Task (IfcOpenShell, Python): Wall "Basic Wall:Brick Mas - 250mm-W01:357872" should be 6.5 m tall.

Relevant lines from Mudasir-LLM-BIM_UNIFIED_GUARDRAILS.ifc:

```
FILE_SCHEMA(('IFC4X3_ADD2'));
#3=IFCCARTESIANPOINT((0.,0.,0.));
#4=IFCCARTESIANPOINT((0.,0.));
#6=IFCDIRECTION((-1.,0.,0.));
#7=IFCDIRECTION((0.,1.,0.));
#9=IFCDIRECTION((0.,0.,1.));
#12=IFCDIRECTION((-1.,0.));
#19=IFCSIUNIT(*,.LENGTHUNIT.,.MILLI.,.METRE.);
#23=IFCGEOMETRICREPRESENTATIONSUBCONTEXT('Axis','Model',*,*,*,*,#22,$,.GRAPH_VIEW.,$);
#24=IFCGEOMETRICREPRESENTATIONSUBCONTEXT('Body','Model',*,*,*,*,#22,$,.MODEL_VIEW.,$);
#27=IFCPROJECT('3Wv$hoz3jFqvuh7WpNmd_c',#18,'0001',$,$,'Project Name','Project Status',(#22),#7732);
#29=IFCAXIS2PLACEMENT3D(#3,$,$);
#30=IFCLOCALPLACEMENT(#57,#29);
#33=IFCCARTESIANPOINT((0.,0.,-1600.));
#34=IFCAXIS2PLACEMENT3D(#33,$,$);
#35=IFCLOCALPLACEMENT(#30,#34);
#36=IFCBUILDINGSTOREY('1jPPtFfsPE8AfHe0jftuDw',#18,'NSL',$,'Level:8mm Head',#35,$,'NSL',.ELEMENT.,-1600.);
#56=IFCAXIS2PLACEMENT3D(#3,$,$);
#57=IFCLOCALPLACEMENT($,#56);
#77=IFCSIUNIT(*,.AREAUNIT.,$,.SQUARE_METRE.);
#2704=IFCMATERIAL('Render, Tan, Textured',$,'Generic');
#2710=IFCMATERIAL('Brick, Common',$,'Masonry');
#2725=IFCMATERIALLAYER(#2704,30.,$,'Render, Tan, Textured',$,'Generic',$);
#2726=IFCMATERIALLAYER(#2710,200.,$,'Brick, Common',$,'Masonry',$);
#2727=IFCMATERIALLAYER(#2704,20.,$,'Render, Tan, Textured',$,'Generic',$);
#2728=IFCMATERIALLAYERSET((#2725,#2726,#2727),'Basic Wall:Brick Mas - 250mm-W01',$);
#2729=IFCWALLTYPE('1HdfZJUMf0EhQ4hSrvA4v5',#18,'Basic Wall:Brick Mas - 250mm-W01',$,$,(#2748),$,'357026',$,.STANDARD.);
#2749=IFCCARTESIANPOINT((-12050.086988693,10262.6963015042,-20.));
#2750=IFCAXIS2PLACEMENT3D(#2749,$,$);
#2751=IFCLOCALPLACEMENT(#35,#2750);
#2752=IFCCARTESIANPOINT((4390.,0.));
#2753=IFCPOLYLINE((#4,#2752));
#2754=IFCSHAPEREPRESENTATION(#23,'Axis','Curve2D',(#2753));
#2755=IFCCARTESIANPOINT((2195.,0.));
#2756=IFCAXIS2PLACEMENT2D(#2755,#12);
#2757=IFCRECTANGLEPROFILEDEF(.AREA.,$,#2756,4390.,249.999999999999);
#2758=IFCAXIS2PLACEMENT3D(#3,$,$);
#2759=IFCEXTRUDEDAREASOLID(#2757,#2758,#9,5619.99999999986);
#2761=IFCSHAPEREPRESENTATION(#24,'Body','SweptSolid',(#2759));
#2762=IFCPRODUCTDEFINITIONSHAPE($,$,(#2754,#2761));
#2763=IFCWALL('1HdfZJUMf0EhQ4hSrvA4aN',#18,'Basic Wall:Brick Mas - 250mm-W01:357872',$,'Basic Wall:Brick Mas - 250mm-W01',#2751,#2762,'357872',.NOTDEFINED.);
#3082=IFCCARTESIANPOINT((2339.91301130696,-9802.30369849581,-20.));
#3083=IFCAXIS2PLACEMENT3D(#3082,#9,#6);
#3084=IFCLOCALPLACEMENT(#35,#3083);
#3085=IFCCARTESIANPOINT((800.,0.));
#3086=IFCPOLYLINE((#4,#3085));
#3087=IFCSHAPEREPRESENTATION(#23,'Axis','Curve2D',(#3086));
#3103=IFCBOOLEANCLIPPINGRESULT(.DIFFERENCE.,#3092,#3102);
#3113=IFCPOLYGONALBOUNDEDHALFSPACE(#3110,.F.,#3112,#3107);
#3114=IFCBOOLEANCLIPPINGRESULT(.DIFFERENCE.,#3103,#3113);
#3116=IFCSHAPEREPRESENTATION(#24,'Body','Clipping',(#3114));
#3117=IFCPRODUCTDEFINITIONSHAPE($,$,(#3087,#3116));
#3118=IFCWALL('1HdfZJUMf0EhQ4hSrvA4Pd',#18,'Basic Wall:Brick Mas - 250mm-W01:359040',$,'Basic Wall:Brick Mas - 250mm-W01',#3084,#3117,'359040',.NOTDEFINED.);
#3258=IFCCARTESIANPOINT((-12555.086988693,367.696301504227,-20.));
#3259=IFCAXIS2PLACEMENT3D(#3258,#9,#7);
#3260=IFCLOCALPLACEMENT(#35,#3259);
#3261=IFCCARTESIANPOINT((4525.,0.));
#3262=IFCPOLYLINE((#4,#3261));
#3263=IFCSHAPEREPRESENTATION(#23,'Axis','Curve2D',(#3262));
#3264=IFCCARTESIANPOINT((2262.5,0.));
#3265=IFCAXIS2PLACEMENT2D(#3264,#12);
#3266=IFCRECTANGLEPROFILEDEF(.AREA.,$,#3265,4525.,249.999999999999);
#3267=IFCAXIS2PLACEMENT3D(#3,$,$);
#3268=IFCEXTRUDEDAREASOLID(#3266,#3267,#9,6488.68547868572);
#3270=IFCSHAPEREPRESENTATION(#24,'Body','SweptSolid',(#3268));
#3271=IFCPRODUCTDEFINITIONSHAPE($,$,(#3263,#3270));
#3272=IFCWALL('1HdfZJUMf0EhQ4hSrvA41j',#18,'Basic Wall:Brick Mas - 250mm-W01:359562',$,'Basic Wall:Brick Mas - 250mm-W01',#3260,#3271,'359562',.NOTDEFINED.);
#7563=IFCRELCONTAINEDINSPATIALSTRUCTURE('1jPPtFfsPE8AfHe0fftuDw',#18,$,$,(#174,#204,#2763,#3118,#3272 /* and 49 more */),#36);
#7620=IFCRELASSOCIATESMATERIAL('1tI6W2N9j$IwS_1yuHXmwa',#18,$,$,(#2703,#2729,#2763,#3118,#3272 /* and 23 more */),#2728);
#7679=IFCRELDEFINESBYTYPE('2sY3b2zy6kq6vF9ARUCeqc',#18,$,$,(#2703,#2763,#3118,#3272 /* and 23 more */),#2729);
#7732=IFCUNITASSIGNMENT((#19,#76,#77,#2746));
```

```python
import ifcopenshell
import ifcopenshell.geom
import ifcopenshell.util.representation
import ifcopenshell.util.shape
import ifcopenshell.util.unit

model = ifcopenshell.open("Mudasir-LLM-BIM_UNIFIED_GUARDRAILS.ifc")
unit_scale = ifcopenshell.util.unit.calculate_unit_scale(model)
settings = ifcopenshell.geom.settings()


def volume(element):
    """Net volume in cubic metres, openings subtracted."""
    shape = ifcopenshell.geom.create_shape(settings, element)
    return ifcopenshell.util.shape.get_volume(shape.geometry)


wall = model.by_id(2763)
before = volume(wall)

body = ifcopenshell.util.representation.get_representation(wall, "Model", "Body")
solid = body.Items[0]
old_height = solid.Depth
solid.Depth = 6.5 / unit_scale
after = volume(wall)

print(f"height {old_height:g} -> {solid.Depth:g}, volume {before:.3f} -> {after:.3f} m3")

model.write("Mudasir-LLM-BIM_UNIFIED_GUARDRAILS-out.ifc")
```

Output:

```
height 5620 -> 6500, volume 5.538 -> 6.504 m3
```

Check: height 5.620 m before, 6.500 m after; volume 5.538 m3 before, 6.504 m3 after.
